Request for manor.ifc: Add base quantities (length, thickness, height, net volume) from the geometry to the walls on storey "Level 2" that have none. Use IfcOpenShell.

First a look at what the model holds.

```python
import ifcopenshell
import ifcopenshell.util.element
import ifcopenshell.util.unit

model = ifcopenshell.open("manor.ifc")
print(model.schema)
for unit_type in ("LENGTHUNIT", "AREAUNIT", "VOLUMEUNIT"):
    print(unit_type, ifcopenshell.util.unit.calculate_unit_scale(model, unit_type))
storey = next(s for s in model.by_type("IfcBuildingStorey") if s.Name == "Level 2")
walls = [e for e in ifcopenshell.util.element.get_decomposition(storey) if e.is_a("IfcWall")]
for e in sorted(walls, key=lambda e: e.id()):
    print(e.id(), e.is_a(), e.Name, list(ifcopenshell.util.element.get_psets(e, qtos_only=True)), sep=" | ")
```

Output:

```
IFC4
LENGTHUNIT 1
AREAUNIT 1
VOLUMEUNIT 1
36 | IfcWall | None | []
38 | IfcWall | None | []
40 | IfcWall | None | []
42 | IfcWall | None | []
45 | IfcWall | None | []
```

```python
import ifcopenshell
import ifcopenshell.api.pset
import ifcopenshell.geom
import ifcopenshell.util.element
import ifcopenshell.util.shape
import ifcopenshell.util.unit

model = ifcopenshell.open("manor.ifc")
unit_scale = ifcopenshell.util.unit.calculate_unit_scale(model)
volume_scale = ifcopenshell.util.unit.calculate_unit_scale(model, "VOLUMEUNIT")
settings = ifcopenshell.geom.settings()

storey = next(s for s in model.by_type("IfcBuildingStorey") if s.Name == "Level 2")
walls = [e for e in ifcopenshell.util.element.get_decomposition(storey) if e.is_a("IfcWall")]

for e in sorted(walls, key=lambda e: e.id()):
    if ifcopenshell.util.element.get_psets(e, qtos_only=True, should_inherit=False):
        continue
    # Geometry comes back in metres, in the element's own axes.
    shape = ifcopenshell.geom.create_shape(settings, e)
    values = {
        "Length": ifcopenshell.util.shape.get_x(shape.geometry) / unit_scale,
        "Width": ifcopenshell.util.shape.get_y(shape.geometry) / unit_scale,
        "Height": ifcopenshell.util.shape.get_z(shape.geometry) / unit_scale,
        "NetVolume": ifcopenshell.util.shape.get_volume(shape.geometry) / volume_scale,
    }
    qto = ifcopenshell.api.pset.add_qto(model, product=e, name="Qto_WallBaseQuantities")
    ifcopenshell.api.pset.edit_qto(model, qto=qto, properties=values)
    print(e.id(), {k: round(v, 3) for k, v in values.items()})

model.write("manor_v2.ifc")
```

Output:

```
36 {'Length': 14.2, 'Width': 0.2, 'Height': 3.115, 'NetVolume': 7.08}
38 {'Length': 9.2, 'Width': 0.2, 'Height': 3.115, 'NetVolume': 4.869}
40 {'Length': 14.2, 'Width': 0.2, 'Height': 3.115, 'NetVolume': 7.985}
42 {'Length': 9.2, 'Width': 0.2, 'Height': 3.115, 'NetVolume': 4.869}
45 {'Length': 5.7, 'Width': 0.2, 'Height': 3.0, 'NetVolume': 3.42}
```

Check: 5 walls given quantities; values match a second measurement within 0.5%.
